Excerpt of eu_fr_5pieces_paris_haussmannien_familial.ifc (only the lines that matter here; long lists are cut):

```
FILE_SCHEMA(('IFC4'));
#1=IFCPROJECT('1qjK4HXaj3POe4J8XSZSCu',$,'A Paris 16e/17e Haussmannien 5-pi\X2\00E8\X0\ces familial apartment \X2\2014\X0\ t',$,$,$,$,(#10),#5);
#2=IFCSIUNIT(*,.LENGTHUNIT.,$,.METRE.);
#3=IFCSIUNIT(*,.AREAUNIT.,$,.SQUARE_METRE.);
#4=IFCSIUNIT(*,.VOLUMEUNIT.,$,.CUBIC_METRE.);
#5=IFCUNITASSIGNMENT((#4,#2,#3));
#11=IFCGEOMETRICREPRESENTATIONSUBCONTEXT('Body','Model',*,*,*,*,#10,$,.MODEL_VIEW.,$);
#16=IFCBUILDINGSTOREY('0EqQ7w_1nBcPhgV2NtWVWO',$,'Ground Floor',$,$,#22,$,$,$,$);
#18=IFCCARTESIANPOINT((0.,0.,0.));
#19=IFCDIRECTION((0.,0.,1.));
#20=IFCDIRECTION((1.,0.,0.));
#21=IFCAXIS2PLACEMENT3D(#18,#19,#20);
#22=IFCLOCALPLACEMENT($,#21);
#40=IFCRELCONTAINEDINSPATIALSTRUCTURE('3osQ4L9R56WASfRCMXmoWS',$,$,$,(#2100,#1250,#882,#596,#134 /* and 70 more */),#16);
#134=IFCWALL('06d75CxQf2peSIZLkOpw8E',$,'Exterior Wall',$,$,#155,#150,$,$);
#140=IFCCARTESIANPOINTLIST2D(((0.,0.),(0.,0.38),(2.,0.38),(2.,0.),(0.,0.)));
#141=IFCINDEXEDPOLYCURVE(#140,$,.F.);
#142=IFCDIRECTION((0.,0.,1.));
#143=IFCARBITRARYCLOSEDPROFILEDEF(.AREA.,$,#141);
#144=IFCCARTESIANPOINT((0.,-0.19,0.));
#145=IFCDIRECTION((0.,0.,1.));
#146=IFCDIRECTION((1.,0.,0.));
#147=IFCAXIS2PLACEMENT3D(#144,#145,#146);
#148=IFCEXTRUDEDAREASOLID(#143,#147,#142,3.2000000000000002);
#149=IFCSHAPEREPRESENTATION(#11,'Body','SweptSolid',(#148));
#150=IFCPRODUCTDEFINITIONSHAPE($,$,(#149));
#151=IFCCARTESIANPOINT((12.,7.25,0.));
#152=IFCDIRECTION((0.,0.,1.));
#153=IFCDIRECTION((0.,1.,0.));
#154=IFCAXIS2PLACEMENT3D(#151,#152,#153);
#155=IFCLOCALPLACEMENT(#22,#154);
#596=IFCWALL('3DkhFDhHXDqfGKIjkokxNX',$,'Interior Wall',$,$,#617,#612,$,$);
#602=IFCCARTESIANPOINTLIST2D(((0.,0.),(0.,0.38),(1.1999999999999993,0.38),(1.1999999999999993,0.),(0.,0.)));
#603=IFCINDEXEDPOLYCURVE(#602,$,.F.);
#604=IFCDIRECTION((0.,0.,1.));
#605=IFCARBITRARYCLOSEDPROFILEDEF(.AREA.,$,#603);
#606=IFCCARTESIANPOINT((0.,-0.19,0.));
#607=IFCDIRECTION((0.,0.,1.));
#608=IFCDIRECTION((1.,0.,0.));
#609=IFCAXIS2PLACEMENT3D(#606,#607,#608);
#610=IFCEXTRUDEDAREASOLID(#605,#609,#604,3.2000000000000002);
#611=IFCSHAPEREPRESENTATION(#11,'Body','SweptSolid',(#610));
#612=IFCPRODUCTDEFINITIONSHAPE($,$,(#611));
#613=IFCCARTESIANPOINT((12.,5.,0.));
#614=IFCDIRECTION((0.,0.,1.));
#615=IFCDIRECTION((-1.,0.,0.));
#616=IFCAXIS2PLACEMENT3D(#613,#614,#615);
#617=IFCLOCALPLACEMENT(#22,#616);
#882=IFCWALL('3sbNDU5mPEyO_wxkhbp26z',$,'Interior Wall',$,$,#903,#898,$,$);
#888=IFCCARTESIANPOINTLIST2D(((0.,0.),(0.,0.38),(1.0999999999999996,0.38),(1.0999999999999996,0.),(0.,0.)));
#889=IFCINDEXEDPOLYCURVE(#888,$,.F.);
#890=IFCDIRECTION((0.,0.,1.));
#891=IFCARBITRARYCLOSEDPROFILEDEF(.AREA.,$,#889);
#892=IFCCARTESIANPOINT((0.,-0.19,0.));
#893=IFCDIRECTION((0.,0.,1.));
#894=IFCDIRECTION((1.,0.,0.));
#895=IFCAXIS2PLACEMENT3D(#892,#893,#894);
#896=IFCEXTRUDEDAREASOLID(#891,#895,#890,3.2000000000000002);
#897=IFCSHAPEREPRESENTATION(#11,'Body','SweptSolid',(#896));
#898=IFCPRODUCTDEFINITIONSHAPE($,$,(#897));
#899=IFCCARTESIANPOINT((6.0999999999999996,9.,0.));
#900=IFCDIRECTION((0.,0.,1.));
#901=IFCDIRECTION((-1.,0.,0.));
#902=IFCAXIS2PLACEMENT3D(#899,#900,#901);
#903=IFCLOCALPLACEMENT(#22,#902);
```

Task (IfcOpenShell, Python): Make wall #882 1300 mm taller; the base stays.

```python
import ifcopenshell
import ifcopenshell.geom
import ifcopenshell.util.representation
import ifcopenshell.util.shape

model = ifcopenshell.open("eu_fr_5pieces_paris_haussmannien_familial.ifc")
settings = ifcopenshell.geom.settings()


def volume(element):
    """Net volume in cubic metres, openings subtracted."""
    shape = ifcopenshell.geom.create_shape(settings, element)
    return ifcopenshell.util.shape.get_volume(shape.geometry)


wall = model.by_id(882)
before = volume(wall)

body = ifcopenshell.util.representation.get_representation(wall, "Model", "Body")
solid = body.Items[0]
old_height = solid.Depth
solid.Depth += 1.3
after = volume(wall)

print(f"height {old_height:g} -> {solid.Depth:g}, volume {before:.3f} -> {after:.3f} m3")

model.write("eu_fr_5pieces_paris_haussmannien_familial_updated.ifc")
```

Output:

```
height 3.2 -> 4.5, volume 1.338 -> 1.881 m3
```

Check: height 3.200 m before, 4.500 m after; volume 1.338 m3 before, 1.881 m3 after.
